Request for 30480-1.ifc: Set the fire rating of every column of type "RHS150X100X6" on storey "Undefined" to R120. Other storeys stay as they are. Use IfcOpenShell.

First a look at what the model holds.

```python
import ifcopenshell
import ifcopenshell.util.element

model = ifcopenshell.open("30480-1.ifc")
print(model.schema)
storey = next(s for s in model.by_type("IfcBuildingStorey") if s.Name == "Undefined")
columns = [e for e in ifcopenshell.util.element.get_decomposition(storey) if e.is_a("IfcColumn")]
seen = {}
for e in columns:
    element_type = ifcopenshell.util.element.get_type(e)
    key = (element_type.Name if element_type != e and element_type else None, ifcopenshell.util.element.get_pset(e, "Pset_ColumnCommon", "FireRating"))
    seen[key] = seen.get(key, 0) + 1
for (name, value), count in sorted(seen.items(), key=str):
    print(count, "x", name, "|", value)
```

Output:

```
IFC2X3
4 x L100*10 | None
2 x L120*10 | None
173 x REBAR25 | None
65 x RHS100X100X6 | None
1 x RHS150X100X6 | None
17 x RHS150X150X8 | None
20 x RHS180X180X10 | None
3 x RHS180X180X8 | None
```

```python
import ifcopenshell
import ifcopenshell.api.pset
import ifcopenshell.util.element

model = ifcopenshell.open("30480-1.ifc")

storey = next(s for s in model.by_type("IfcBuildingStorey") if s.Name == "Undefined")
columns = [e for e in ifcopenshell.util.element.get_decomposition(storey) if e.is_a("IfcColumn")]

count = 0
for e in columns:
    element_type = ifcopenshell.util.element.get_type(e)
    if element_type in (None, e) or element_type.Name != "RHS150X100X6":
        continue
    # add_pset returns the element's existing set when there is one.
    pset = ifcopenshell.api.pset.add_pset(model, product=e, name="Pset_ColumnCommon")
    ifcopenshell.api.pset.edit_pset(model, pset=pset, properties={"FireRating": "R120"})
    count += 1

print(count, "columns updated")

model.write("30480-1_rev.ifc")
```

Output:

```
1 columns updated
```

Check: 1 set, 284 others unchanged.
